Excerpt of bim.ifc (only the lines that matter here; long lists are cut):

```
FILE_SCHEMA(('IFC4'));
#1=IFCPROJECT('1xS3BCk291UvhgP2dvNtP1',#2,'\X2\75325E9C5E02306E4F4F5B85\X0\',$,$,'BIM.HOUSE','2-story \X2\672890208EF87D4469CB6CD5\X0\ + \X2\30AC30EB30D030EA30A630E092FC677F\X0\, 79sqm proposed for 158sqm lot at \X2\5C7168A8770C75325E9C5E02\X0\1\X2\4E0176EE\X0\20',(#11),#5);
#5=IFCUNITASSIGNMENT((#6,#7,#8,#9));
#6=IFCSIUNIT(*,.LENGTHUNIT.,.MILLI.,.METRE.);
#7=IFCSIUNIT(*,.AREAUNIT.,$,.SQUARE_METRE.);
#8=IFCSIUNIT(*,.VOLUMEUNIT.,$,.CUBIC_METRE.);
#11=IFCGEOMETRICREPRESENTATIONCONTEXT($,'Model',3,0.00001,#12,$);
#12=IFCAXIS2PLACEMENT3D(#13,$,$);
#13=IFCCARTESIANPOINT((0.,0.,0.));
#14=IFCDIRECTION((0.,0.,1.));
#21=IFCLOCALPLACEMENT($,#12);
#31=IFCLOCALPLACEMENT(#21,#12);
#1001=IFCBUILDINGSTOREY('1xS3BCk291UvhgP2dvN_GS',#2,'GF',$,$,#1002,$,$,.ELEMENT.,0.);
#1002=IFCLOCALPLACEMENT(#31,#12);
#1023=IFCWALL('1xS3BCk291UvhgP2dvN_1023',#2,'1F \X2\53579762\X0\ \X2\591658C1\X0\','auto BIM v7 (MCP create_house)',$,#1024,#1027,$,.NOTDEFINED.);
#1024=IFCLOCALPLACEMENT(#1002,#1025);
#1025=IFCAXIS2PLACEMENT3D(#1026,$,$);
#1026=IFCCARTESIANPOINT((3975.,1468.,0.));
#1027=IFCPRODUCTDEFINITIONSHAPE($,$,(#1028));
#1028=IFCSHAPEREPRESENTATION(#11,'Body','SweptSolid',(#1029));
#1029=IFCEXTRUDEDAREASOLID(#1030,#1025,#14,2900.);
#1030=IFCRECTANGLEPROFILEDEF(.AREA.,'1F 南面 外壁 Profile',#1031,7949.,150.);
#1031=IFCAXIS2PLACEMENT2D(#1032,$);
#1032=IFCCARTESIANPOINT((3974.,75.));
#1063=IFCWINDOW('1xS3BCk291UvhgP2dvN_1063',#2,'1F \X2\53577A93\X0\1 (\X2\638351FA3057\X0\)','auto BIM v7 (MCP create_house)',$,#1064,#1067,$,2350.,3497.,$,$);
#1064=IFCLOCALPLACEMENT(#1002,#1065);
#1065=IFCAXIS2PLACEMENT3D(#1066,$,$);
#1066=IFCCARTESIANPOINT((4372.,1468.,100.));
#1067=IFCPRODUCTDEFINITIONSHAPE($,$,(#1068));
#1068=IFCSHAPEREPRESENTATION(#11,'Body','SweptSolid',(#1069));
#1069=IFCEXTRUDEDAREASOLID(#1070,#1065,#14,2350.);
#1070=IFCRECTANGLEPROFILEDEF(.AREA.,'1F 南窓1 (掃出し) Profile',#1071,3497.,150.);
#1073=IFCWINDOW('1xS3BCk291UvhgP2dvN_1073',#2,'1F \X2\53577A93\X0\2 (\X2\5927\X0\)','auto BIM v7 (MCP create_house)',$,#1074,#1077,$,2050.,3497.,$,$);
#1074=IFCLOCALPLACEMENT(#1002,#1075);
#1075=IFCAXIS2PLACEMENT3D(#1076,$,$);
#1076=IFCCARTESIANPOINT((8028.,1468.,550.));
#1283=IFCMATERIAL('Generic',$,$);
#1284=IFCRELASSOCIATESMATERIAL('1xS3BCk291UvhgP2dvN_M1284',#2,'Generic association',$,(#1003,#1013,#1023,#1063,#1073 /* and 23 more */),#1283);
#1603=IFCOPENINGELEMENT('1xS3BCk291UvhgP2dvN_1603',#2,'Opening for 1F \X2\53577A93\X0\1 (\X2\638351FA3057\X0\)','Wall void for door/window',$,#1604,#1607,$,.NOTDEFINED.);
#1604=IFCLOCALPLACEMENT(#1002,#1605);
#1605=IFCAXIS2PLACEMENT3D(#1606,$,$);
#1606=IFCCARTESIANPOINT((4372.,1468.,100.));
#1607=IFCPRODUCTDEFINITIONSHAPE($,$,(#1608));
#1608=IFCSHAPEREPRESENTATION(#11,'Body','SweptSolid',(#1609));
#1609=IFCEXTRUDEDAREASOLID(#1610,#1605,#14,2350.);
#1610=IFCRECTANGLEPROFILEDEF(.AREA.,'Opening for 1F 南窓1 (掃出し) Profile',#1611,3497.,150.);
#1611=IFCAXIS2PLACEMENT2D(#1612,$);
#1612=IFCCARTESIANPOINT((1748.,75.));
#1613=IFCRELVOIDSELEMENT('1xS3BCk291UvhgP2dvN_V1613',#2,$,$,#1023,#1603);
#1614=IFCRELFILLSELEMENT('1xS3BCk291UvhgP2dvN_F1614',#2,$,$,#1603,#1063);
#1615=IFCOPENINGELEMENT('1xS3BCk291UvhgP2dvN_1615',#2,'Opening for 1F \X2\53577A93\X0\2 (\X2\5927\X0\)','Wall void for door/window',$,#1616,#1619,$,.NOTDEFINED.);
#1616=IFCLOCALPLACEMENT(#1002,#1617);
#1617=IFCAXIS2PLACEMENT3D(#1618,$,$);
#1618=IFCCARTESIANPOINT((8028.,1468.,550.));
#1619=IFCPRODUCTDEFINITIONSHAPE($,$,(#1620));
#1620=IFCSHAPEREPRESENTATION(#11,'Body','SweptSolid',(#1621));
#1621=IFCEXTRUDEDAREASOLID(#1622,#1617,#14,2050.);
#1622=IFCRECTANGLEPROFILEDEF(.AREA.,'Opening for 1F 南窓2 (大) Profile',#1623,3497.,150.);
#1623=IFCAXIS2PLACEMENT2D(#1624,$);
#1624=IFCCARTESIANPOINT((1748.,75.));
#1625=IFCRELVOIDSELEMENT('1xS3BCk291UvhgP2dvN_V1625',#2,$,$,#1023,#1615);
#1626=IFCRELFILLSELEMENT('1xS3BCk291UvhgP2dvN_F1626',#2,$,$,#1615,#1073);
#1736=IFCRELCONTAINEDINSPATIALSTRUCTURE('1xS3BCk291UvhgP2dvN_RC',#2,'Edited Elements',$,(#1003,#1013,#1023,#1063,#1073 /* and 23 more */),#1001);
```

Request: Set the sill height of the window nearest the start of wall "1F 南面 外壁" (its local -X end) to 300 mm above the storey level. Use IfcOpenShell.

```python
import numpy as np
import ifcopenshell
import ifcopenshell.api.geometry
import ifcopenshell.geom
import ifcopenshell.util.element
import ifcopenshell.util.placement
import ifcopenshell.util.shape
import ifcopenshell.util.unit

model = ifcopenshell.open("bim.ifc")
unit_scale = ifcopenshell.util.unit.calculate_unit_scale(model)

window = model.by_guid("1xS3BCk291UvhgP2dvN_1063")
opening = window.FillsVoids[0].RelatingOpeningElement
storey = ifcopenshell.util.element.get_container(window, ifc_class="IfcBuildingStorey")
level = ifcopenshell.util.placement.get_local_placement(storey.ObjectPlacement)[2, 3]

# The opening's origin need not be at the sill, so measure its lowest point.
shape = ifcopenshell.geom.create_shape(ifcopenshell.geom.settings(), opening)
bottom = ifcopenshell.util.shape.get_shape_bottom_elevation(shape, shape.geometry) / unit_scale
dz = level + 0.3 / unit_scale - bottom

shift = np.array([0.0, 0.0, dz])
# The window is not placed relative to its opening, so move both.
for product in (opening, window):
    matrix = ifcopenshell.util.placement.get_local_placement(product.ObjectPlacement)
    matrix[:3, 3] += shift
    ifcopenshell.api.geometry.edit_object_placement(model, product=product, matrix=matrix, is_si=False)

print(f"moved by {dz * unit_scale:+.3f} m")

model.write("bim-out.ifc")
```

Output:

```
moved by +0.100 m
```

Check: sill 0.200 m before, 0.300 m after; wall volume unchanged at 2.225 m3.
